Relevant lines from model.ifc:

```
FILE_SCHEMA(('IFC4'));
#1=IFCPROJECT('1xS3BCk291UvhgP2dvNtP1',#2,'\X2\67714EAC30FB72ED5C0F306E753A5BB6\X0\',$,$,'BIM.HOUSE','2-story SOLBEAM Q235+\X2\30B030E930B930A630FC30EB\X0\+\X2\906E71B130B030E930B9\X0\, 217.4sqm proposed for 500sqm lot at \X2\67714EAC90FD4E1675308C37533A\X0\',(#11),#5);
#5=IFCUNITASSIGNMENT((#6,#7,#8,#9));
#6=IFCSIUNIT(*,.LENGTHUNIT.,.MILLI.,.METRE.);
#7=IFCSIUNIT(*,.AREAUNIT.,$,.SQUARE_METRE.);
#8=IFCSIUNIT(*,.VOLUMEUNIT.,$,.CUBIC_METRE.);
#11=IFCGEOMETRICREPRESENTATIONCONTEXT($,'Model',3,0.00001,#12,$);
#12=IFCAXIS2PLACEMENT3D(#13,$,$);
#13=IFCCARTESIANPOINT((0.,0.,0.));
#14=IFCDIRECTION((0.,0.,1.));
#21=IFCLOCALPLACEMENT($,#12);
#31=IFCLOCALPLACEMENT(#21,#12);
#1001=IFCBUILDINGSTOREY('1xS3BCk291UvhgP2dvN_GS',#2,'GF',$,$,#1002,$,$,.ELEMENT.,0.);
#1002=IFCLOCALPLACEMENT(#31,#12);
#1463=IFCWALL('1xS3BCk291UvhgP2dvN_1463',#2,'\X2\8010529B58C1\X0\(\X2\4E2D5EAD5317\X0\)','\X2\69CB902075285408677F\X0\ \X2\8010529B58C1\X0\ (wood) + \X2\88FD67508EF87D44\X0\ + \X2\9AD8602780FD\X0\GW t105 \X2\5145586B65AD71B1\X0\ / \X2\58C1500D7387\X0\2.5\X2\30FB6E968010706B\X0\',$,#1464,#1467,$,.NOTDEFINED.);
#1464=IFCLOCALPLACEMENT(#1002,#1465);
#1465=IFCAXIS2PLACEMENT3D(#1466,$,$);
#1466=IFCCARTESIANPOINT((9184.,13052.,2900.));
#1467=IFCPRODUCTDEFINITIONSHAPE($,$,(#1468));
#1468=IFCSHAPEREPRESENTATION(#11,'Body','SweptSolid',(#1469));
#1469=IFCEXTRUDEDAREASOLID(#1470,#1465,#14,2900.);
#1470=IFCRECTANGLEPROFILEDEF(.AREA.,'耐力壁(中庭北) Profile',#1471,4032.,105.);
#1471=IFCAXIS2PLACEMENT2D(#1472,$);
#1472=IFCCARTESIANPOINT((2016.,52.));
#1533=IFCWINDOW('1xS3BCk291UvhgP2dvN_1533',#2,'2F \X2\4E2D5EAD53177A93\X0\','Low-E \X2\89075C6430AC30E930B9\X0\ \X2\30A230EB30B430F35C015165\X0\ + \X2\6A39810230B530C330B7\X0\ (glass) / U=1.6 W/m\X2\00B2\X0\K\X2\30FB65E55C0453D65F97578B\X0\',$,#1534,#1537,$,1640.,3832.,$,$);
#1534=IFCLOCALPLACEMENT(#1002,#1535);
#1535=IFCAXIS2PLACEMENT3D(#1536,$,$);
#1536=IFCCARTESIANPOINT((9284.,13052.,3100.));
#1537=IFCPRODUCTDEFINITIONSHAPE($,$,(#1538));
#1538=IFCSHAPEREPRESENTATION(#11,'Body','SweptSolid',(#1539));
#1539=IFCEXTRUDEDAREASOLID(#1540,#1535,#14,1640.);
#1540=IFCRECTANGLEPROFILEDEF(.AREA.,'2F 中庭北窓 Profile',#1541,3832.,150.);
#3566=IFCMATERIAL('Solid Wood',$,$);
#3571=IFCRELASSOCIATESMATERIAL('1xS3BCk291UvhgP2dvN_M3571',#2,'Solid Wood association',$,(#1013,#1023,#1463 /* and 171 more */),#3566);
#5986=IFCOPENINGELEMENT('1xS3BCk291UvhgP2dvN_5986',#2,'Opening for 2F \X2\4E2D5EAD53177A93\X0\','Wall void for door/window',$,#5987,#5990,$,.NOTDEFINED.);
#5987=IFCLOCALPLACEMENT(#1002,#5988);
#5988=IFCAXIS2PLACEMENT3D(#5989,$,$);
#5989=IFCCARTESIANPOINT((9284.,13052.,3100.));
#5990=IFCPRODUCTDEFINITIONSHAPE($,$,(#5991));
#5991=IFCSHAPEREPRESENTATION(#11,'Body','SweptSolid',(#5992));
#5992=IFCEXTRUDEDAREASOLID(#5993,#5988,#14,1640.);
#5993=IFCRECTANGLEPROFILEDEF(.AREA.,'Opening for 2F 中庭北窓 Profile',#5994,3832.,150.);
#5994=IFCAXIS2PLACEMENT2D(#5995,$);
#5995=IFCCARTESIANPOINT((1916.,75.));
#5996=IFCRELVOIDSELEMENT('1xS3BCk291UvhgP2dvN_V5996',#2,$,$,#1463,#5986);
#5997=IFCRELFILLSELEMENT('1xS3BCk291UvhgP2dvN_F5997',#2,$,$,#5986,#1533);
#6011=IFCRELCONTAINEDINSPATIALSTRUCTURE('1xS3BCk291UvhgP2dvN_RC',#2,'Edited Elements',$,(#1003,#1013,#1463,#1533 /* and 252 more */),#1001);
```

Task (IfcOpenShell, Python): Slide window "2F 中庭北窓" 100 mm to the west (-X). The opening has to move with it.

```python
import ifcopenshell
import ifcopenshell.api.geometry
import ifcopenshell.util.placement
import ifcopenshell.util.unit

model = ifcopenshell.open("model.ifc")
unit_scale = ifcopenshell.util.unit.calculate_unit_scale(model)

window = model.by_guid("1xS3BCk291UvhgP2dvN_1533")
opening = window.FillsVoids[0].RelatingOpeningElement
wall = opening.VoidsElements[0].RelatingBuildingElement

wall_matrix = ifcopenshell.util.placement.get_local_placement(wall.ObjectPlacement)
shift = wall_matrix[:3, 0] * -0.1 / unit_scale
before = ifcopenshell.util.placement.get_local_placement(window.ObjectPlacement)[:3, 3].copy()

# The window is not placed relative to its opening, so move both.
for product in (opening, window):
    matrix = ifcopenshell.util.placement.get_local_placement(product.ObjectPlacement)
    matrix[:3, 3] += shift
    ifcopenshell.api.geometry.edit_object_placement(model, product=product, matrix=matrix, is_si=False)

after = ifcopenshell.util.placement.get_local_placement(window.ObjectPlacement)[:3, 3]
print("window moved by", (after - before).round(3) + 0.0)

model.write("model-out.ifc")
```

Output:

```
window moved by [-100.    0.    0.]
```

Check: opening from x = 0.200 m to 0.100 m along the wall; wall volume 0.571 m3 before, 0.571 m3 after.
